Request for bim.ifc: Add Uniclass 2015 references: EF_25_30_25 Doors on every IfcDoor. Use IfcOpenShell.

First a look at what the model holds.

```python
import ifcopenshell

model = ifcopenshell.open("bim.ifc")
print(model.schema)
print("classifications:", [c.Name for c in model.by_type("IfcClassification")])
for ifc_class in ("IfcDoor", "IfcRoof", "IfcStair", "IfcWall", "IfcWindow"):
    print(ifc_class, len(model.by_type(ifc_class)))
```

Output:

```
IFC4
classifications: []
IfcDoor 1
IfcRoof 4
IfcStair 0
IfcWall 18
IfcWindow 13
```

```python
import ifcopenshell
import ifcopenshell.api.classification

model = ifcopenshell.open("bim.ifc")

system = ifcopenshell.api.classification.add_classification(model, classification="Uniclass 2015")

codes = {
    "IfcDoor": ("EF_25_30_25", "Doors"),
}
for ifc_class, (code, name) in codes.items():
    products = model.by_type(ifc_class)
    ifcopenshell.api.classification.add_reference(
        model, products=products, classification=system, identification=code, name=name
    )
    print(code, len(products))

model.write("bim_rev.ifc")
```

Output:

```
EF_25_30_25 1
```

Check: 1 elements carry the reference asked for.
